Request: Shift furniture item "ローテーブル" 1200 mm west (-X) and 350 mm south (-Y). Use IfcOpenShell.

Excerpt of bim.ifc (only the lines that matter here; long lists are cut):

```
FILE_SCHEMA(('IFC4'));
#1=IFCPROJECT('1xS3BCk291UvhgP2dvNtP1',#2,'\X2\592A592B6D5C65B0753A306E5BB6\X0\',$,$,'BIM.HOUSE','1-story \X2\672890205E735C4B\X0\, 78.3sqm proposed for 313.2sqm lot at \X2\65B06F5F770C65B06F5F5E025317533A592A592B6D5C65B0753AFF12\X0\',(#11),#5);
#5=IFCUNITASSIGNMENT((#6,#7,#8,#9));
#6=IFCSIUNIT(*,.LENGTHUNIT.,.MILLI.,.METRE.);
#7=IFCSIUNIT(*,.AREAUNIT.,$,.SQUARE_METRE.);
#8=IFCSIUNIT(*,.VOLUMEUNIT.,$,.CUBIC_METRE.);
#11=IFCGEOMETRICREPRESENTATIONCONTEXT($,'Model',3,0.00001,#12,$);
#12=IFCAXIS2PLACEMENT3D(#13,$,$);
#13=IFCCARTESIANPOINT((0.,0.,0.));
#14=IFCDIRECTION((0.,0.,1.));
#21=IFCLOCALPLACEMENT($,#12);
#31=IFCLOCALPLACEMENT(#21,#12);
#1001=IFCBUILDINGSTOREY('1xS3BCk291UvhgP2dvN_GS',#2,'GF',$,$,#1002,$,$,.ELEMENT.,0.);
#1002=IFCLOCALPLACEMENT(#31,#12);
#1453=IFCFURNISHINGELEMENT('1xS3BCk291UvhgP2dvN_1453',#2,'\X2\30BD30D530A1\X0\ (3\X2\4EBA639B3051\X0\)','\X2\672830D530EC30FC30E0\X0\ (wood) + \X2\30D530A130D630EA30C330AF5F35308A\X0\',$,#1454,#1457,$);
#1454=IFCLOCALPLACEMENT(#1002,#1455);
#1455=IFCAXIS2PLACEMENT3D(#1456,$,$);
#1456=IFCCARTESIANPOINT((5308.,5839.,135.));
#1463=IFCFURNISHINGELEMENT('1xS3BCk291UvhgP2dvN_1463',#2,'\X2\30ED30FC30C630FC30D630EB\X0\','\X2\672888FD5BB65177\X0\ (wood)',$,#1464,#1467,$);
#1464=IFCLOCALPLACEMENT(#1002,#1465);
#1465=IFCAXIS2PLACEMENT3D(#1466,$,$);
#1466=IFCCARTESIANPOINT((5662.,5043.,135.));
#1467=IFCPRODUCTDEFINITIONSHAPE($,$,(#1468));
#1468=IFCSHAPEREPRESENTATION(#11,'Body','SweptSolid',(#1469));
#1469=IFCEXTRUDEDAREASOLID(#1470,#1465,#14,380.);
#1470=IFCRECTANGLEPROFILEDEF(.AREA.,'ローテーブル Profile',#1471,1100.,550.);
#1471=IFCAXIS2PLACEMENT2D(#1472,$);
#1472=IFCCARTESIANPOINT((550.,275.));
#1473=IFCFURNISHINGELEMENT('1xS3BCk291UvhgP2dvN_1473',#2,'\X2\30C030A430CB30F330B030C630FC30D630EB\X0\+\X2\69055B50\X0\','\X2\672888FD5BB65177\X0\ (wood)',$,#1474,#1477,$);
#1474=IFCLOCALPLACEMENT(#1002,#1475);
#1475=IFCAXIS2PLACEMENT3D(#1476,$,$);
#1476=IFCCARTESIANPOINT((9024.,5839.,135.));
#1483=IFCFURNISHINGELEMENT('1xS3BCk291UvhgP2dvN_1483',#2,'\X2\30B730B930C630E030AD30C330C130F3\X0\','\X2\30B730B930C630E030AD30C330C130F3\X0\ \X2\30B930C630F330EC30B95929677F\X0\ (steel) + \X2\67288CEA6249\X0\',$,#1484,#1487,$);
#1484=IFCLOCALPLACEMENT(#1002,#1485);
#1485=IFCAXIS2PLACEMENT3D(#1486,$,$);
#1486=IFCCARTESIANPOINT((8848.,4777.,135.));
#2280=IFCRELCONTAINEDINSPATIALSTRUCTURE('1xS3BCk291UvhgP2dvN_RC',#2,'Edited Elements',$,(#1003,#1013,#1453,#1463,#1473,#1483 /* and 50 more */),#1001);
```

```python
import ifcopenshell
import ifcopenshell.api.geometry
import ifcopenshell.util.placement
import ifcopenshell.util.unit

model = ifcopenshell.open("bim.ifc")
unit_scale = ifcopenshell.util.unit.calculate_unit_scale(model)

item = model.by_id(1463)
matrix = ifcopenshell.util.placement.get_local_placement(item.ObjectPlacement)
matrix[0, 3] -= 1.2 / unit_scale
matrix[1, 3] -= 0.35 / unit_scale
ifcopenshell.api.geometry.edit_object_placement(model, product=item, matrix=matrix, is_si=False)

print(ifcopenshell.util.placement.get_local_placement(item.ObjectPlacement).round(3) + 0.0)

model.write("bim_edited.ifc")
```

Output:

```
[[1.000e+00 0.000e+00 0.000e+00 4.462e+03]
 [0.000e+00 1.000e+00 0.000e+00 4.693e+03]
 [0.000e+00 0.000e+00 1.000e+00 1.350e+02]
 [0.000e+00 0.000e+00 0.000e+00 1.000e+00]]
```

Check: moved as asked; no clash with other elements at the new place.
